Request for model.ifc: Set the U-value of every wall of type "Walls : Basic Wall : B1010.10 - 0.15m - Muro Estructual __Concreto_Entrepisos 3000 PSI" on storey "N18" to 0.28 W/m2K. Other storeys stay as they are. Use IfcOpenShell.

First a look at what the model holds.

```python
import ifcopenshell
import ifcopenshell.util.element

model = ifcopenshell.open("model.ifc")
print(model.schema)
storey = next(s for s in model.by_type("IfcBuildingStorey") if s.Name == "N18")
walls = [e for e in ifcopenshell.util.element.get_decomposition(storey) if e.is_a("IfcWall")]
seen = {}
for e in walls:
    element_type = ifcopenshell.util.element.get_type(e)
    key = (element_type.Name if element_type != e and element_type else None, ifcopenshell.util.element.get_pset(e, "Pset_WallCommon", "ThermalTransmittance"))
    seen[key] = seen.get(key, 0) + 1
for (name, value), count in sorted(seen.items(), key=str):
    print(count, "x", name, "|", value)
```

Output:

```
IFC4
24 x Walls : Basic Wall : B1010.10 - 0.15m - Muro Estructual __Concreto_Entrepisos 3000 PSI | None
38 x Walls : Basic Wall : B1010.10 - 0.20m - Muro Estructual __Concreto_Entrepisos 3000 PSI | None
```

```python
import ifcopenshell
import ifcopenshell.api.pset
import ifcopenshell.util.element

model = ifcopenshell.open("model.ifc")

storey = next(s for s in model.by_type("IfcBuildingStorey") if s.Name == "N18")
walls = [e for e in ifcopenshell.util.element.get_decomposition(storey) if e.is_a("IfcWall")]

count = 0
for e in walls:
    element_type = ifcopenshell.util.element.get_type(e)
    if element_type in (None, e) or element_type.Name != "Walls : Basic Wall : B1010.10 - 0.15m - Muro Estructual __Concreto_Entrepisos 3000 PSI":
        continue
    # add_pset returns the element's existing set when there is one.
    pset = ifcopenshell.api.pset.add_pset(model, product=e, name="Pset_WallCommon")
    ifcopenshell.api.pset.edit_pset(model, pset=pset, properties={"ThermalTransmittance": 0.28})
    count += 1

print(count, "walls updated")

model.write("model_updated.ifc")
```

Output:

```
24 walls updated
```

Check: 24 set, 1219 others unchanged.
